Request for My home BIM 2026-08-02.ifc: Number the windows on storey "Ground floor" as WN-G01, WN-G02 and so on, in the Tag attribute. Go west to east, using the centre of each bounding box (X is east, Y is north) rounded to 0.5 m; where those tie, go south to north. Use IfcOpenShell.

First a look at what the model holds.

```python
import ifcopenshell
import ifcopenshell.util.element
import ifcopenshell.util.placement

model = ifcopenshell.open("My home BIM 2026-08-02.ifc")
print(model.schema)
storey = next(s for s in model.by_type("IfcBuildingStorey") if s.Name == "Ground floor")
windows = [e for e in ifcopenshell.util.element.get_decomposition(storey) if e.is_a("IfcWindow")]
for e in sorted(windows, key=lambda e: e.id()):
    origin = ifcopenshell.util.placement.get_local_placement(e.ObjectPlacement)[:3, 3]
    print(e.id(), e.Tag, e.Name, origin.round(2) + 0.0, sep=" | ")
```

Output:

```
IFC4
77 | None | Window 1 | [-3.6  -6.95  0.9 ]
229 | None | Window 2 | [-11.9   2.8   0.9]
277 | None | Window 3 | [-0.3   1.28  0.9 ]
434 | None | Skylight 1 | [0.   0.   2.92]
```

```python
import ifcopenshell
import ifcopenshell.geom
import ifcopenshell.util.element
import ifcopenshell.util.shape

model = ifcopenshell.open("My home BIM 2026-08-02.ifc")
settings = ifcopenshell.geom.settings()
settings.set("use-world-coords", True)


def centre(element):
    shape = ifcopenshell.geom.create_shape(settings, element)
    return ifcopenshell.util.shape.get_bbox_centroid(shape.geometry)


storey = next(s for s in model.by_type("IfcBuildingStorey") if s.Name == "Ground floor")
windows = [e for e in ifcopenshell.util.element.get_decomposition(storey) if e.is_a("IfcWindow")]

# Insertion points can sit at a corner or the storey origin, so sort by the geometry (in metres).
centres = {e: centre(e) for e in windows}
windows.sort(key=lambda e: (round(centres[e][0] / 0.5), centres[e][1]))

for i, e in enumerate(windows, start=1):
    number = f"WN-G{i:02d}"
    e.Tag = number
    print(e.id(), number)

model.write("My home BIM 2026-08-02_edited.ifc")
```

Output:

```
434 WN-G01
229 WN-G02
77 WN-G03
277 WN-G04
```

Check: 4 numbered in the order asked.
